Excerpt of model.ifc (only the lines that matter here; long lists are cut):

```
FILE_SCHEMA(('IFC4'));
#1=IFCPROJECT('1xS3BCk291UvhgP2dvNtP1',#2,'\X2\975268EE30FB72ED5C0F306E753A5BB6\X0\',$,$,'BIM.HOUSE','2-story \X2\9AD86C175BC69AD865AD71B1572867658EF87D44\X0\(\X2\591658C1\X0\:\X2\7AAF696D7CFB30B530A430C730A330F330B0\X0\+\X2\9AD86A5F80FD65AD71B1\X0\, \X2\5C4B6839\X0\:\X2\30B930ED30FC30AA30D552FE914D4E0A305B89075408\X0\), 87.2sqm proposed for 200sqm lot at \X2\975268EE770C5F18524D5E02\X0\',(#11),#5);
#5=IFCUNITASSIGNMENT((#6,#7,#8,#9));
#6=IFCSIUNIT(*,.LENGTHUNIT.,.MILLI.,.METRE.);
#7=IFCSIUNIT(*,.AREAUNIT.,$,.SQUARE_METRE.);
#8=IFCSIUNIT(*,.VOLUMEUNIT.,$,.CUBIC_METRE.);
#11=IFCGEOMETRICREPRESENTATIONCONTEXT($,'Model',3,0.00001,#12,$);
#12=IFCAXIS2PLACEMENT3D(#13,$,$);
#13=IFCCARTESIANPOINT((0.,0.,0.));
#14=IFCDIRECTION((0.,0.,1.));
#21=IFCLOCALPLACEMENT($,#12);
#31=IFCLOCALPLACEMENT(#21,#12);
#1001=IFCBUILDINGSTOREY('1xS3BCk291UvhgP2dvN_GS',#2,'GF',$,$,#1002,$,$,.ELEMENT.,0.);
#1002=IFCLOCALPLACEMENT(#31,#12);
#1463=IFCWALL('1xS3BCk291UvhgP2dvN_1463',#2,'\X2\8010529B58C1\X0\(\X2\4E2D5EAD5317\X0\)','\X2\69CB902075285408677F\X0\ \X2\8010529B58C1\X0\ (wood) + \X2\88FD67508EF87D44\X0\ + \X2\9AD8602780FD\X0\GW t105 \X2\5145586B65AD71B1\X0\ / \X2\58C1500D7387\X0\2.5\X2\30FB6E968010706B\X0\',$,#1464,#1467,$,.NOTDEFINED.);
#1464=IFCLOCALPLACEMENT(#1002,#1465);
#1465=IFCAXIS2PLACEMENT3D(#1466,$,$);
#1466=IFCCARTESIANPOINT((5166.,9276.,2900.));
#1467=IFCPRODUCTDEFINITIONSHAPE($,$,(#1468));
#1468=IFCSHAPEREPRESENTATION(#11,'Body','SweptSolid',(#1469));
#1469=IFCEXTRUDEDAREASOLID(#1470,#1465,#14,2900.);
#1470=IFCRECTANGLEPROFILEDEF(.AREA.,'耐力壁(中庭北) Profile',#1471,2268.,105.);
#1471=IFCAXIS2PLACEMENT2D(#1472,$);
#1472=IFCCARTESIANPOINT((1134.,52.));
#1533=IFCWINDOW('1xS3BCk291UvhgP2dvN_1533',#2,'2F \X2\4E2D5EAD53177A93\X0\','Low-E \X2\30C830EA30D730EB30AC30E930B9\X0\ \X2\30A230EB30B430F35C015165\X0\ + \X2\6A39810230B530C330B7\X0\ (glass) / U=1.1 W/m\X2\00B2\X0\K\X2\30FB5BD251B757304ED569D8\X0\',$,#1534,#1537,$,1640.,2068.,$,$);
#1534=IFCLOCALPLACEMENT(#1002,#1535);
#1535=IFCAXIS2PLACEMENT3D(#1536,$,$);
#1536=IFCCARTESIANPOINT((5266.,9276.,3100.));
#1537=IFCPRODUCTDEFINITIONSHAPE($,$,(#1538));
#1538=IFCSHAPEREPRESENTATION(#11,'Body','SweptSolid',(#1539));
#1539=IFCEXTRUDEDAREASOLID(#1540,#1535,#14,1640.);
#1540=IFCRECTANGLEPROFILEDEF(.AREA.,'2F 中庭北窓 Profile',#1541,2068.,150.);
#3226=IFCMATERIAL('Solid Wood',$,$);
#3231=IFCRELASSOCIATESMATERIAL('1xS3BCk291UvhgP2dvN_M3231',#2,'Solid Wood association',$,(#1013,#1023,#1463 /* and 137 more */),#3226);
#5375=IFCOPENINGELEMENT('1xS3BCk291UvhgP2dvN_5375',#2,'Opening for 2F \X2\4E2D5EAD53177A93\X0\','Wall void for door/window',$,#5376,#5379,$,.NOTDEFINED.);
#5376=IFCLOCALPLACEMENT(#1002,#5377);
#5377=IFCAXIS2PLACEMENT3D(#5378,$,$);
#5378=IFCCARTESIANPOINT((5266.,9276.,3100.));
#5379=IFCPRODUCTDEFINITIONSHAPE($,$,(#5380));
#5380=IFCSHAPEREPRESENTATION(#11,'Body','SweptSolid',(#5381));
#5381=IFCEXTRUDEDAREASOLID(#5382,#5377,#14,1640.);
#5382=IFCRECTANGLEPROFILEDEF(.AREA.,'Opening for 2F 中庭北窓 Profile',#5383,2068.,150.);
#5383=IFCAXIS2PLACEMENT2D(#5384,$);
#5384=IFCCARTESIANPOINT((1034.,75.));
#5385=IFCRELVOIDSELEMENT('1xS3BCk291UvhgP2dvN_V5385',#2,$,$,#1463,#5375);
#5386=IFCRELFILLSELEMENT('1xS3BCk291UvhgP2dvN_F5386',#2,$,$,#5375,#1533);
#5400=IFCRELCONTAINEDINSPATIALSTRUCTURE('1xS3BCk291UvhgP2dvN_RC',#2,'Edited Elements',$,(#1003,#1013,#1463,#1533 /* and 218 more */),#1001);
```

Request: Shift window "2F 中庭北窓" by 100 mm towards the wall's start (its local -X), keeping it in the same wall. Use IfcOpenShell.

```python
import ifcopenshell
import ifcopenshell.api.geometry
import ifcopenshell.util.placement

model = ifcopenshell.open("model.ifc")

window = model.by_guid("1xS3BCk291UvhgP2dvN_1533")
opening = window.FillsVoids[0].RelatingOpeningElement
wall = opening.VoidsElements[0].RelatingBuildingElement

wall_matrix = ifcopenshell.util.placement.get_local_placement(wall.ObjectPlacement)
shift = wall_matrix[:3, 0] * -100.0
before = ifcopenshell.util.placement.get_local_placement(window.ObjectPlacement)[:3, 3].copy()

# The window is not placed relative to its opening, so move both.
for product in (opening, window):
    matrix = ifcopenshell.util.placement.get_local_placement(product.ObjectPlacement)
    matrix[:3, 3] += shift
    ifcopenshell.api.geometry.edit_object_placement(model, product=product, matrix=matrix, is_si=False)

after = ifcopenshell.util.placement.get_local_placement(window.ObjectPlacement)[:3, 3]
print("window moved by", (after - before).round(3) + 0.0)

model.write("model-out.ifc")
```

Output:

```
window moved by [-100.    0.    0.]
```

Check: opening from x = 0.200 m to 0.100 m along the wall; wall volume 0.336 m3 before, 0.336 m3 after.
